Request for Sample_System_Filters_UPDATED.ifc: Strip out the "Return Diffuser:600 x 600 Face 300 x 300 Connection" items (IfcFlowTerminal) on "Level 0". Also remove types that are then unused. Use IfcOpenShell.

First a look at what the model holds.

```python
import ifcopenshell
import ifcopenshell.util.element

model = ifcopenshell.open("Sample_System_Filters_UPDATED.ifc")
print(model.schema)
storey = next(s for s in model.by_type("IfcBuildingStorey") if s.Name == "Level 0")
terminals = [e for e in ifcopenshell.util.element.get_decomposition(storey) if e.is_a("IfcFlowTerminal")]
seen = {}
for e in terminals:
    element_type = ifcopenshell.util.element.get_type(e)
    name = element_type.Name if element_type not in (None, e) else None
    seen[name] = seen.get(name, 0) + 1
for name, count in sorted(seen.items(), key=str):
    print(count, "x", name)
```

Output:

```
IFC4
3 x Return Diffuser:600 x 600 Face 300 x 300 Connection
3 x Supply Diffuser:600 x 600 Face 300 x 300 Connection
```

```python
import ifcopenshell
import ifcopenshell.api.root
import ifcopenshell.util.element

model = ifcopenshell.open("Sample_System_Filters_UPDATED.ifc")

storey = next(s for s in model.by_type("IfcBuildingStorey") if s.Name == "Level 0")
terminals = [e for e in ifcopenshell.util.element.get_decomposition(storey) if e.is_a("IfcFlowTerminal")]
targets = [e for e in terminals if (t := ifcopenshell.util.element.get_type(e)) not in (None, e) and t.Name == "Return Diffuser:600 x 600 Face 300 x 300 Connection"]
types = {ifcopenshell.util.element.get_type(e) for e in targets} - {None, *targets}

for e in targets:
    ifcopenshell.api.root.remove_product(model, product=e)
print(len(targets), "removed")

unused = [t for t in types if not ifcopenshell.util.element.get_types(t)]
for t in unused:
    ifcopenshell.api.root.remove_product(model, product=t)
print(len(unused), "unused types removed")

model.write("Sample_System_Filters_UPDATED-out.ifc")
```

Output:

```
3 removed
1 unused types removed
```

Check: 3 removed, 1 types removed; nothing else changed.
